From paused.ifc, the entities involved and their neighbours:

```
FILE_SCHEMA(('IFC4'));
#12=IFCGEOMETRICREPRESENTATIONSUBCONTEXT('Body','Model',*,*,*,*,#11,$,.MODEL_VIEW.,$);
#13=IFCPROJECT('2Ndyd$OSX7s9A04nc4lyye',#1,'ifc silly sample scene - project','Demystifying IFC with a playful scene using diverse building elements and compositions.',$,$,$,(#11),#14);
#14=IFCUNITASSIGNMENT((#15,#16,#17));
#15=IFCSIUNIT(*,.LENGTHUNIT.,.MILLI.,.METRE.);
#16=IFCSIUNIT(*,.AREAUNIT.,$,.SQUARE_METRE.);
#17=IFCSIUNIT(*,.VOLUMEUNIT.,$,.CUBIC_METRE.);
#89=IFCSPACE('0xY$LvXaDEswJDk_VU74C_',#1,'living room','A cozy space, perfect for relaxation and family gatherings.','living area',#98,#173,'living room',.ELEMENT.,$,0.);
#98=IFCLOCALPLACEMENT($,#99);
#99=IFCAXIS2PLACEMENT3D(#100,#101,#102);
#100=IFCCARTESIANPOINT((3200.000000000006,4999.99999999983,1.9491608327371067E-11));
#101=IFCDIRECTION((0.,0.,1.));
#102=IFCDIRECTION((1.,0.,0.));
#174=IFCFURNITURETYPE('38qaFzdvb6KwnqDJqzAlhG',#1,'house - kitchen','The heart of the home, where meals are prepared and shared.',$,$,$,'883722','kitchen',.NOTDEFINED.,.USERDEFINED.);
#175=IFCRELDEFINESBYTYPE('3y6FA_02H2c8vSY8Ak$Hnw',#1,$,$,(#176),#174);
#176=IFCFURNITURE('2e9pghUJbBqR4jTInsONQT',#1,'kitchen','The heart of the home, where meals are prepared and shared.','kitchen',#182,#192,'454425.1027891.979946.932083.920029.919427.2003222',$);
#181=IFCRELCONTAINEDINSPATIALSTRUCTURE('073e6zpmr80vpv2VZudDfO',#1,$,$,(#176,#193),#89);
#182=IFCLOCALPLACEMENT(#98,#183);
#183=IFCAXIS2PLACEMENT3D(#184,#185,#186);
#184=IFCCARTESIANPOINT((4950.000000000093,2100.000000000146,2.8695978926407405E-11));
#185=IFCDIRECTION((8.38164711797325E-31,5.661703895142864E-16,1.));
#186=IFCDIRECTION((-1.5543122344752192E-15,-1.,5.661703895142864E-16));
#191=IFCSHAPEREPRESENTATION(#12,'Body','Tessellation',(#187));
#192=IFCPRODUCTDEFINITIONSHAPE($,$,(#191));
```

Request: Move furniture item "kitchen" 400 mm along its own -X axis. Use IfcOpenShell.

```python
import ifcopenshell
import ifcopenshell.api.geometry
import ifcopenshell.util.placement
import ifcopenshell.util.unit

model = ifcopenshell.open("paused.ifc")
unit_scale = ifcopenshell.util.unit.calculate_unit_scale(model)

item = model.by_guid("2e9pghUJbBqR4jTInsONQT")
matrix = ifcopenshell.util.placement.get_local_placement(item.ObjectPlacement)
matrix[:3, 3] -= matrix[:3, 0] * 0.4 / unit_scale
ifcopenshell.api.geometry.edit_object_placement(model, product=item, matrix=matrix, is_si=False)

print(ifcopenshell.util.placement.get_local_placement(item.ObjectPlacement).round(3) + 0.0)

model.write("paused-out.ifc")
```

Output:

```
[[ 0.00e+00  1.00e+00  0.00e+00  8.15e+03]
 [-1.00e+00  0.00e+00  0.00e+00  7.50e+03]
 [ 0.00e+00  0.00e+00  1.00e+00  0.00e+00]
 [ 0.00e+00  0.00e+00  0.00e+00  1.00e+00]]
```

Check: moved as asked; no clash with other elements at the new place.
